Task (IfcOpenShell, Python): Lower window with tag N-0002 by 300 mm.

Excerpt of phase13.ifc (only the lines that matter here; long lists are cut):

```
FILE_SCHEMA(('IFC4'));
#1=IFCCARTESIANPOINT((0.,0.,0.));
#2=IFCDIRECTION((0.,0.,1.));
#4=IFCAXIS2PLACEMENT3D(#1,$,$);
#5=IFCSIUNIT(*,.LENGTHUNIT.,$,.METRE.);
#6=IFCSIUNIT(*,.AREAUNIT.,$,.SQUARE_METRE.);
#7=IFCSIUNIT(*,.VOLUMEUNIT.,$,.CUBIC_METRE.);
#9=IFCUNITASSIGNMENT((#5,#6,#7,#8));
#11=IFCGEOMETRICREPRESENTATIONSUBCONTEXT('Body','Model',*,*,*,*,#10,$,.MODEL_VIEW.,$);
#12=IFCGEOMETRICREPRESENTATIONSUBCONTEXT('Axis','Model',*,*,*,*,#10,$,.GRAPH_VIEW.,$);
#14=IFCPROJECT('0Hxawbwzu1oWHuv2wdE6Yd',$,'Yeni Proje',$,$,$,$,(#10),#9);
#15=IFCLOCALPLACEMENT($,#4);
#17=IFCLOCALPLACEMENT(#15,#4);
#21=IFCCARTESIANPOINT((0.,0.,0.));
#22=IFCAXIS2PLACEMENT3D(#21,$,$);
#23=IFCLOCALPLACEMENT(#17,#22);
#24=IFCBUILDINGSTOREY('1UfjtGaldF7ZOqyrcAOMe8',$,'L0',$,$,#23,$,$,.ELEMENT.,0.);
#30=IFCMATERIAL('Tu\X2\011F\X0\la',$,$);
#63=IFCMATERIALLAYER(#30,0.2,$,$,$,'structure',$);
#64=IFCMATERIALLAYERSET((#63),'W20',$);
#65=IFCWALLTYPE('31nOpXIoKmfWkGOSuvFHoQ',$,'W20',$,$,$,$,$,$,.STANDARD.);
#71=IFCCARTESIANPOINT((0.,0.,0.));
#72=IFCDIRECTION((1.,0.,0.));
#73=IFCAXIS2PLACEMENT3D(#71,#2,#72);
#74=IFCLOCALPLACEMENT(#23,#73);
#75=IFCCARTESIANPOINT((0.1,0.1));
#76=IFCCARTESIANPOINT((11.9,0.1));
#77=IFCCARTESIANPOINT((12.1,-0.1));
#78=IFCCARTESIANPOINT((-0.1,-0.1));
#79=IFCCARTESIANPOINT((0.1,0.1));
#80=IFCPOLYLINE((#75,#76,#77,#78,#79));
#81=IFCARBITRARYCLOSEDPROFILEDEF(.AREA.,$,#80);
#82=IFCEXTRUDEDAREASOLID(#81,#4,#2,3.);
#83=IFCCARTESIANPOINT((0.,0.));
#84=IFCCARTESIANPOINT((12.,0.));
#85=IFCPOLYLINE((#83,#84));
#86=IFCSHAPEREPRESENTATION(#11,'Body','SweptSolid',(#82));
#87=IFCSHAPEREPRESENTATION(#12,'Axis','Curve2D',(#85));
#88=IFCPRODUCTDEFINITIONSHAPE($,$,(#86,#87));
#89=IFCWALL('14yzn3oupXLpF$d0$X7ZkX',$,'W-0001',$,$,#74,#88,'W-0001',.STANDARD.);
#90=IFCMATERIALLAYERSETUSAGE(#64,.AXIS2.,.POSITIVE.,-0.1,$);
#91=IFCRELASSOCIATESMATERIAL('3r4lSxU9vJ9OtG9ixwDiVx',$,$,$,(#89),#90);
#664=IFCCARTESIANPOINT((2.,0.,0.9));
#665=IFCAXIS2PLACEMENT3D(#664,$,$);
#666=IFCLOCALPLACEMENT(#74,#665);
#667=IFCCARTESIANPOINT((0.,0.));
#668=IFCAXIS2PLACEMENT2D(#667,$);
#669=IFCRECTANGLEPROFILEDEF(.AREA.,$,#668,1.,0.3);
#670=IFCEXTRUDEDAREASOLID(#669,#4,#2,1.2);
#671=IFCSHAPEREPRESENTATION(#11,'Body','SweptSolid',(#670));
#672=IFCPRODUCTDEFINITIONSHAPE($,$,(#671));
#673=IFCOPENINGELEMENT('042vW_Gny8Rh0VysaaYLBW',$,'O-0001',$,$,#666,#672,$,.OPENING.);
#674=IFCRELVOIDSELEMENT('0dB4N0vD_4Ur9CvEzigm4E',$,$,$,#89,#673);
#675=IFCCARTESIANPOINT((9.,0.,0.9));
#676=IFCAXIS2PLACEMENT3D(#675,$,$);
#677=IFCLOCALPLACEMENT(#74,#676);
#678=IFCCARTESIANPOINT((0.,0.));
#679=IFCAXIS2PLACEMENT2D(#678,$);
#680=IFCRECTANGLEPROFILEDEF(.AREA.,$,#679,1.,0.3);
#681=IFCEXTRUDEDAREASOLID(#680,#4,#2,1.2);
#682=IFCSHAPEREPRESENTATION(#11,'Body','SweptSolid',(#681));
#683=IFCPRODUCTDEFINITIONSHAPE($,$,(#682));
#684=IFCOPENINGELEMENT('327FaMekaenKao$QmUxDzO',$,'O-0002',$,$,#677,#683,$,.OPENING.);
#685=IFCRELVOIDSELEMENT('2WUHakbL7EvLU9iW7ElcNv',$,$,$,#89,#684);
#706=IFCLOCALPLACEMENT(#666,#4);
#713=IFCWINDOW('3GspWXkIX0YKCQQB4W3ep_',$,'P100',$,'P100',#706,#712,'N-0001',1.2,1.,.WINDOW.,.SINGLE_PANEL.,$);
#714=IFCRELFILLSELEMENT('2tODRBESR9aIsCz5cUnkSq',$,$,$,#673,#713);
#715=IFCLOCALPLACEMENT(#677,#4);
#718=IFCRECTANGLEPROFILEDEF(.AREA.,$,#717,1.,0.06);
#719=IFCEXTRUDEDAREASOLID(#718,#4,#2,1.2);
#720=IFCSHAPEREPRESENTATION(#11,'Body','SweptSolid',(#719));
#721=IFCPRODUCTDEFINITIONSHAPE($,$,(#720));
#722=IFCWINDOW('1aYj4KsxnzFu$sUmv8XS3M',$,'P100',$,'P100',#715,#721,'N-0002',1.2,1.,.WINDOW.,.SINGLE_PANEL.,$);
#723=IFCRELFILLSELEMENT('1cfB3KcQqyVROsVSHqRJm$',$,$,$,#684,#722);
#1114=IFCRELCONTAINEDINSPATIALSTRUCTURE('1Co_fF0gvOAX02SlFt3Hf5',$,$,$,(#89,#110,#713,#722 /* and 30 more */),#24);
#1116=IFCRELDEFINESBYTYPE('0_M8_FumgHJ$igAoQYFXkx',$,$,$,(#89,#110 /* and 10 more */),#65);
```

```python
import numpy as np
import ifcopenshell
import ifcopenshell.api.geometry
import ifcopenshell.util.placement
import ifcopenshell.util.unit

model = ifcopenshell.open("phase13.ifc")
unit_scale = ifcopenshell.util.unit.calculate_unit_scale(model)

window = model.by_id(722)
opening = window.FillsVoids[0].RelatingOpeningElement
dz = -0.3 / unit_scale

shift = np.array([0.0, 0.0, dz])
# The window is placed relative to its opening, so it follows when the opening moves.
matrix = ifcopenshell.util.placement.get_local_placement(opening.ObjectPlacement)
matrix[:3, 3] += shift
ifcopenshell.api.geometry.edit_object_placement(
    model, product=opening, matrix=matrix, is_si=False, should_transform_children=True
)

print(f"moved by {dz * unit_scale:+.3f} m")

model.write("phase13-out.ifc")
```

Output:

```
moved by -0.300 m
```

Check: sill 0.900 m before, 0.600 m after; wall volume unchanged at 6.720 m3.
